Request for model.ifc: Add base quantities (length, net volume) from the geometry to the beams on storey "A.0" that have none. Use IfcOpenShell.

First a look at what the model holds.

```python
import ifcopenshell
import ifcopenshell.util.element
import ifcopenshell.util.unit

model = ifcopenshell.open("model.ifc")
print(model.schema)
for unit_type in ("LENGTHUNIT", "AREAUNIT", "VOLUMEUNIT"):
    print(unit_type, ifcopenshell.util.unit.calculate_unit_scale(model, unit_type))
storey = next(s for s in model.by_type("IfcBuildingStorey") if s.Name == "A.0")
beams = [e for e in ifcopenshell.util.element.get_decomposition(storey) if e.is_a("IfcBeam")]
for e in sorted(beams, key=lambda e: e.id()):
    print(e.id(), e.is_a(), e.Name, list(ifcopenshell.util.element.get_psets(e, qtos_only=True)), sep=" | ")
```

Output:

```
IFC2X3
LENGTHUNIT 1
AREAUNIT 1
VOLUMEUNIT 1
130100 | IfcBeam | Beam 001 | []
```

```python
import ifcopenshell
import ifcopenshell.api.pset
import ifcopenshell.geom
import ifcopenshell.util.element
import ifcopenshell.util.shape
import ifcopenshell.util.unit

model = ifcopenshell.open("model.ifc")
unit_scale = ifcopenshell.util.unit.calculate_unit_scale(model)
volume_scale = ifcopenshell.util.unit.calculate_unit_scale(model, "VOLUMEUNIT")
settings = ifcopenshell.geom.settings()

storey = next(s for s in model.by_type("IfcBuildingStorey") if s.Name == "A.0")
beams = [e for e in ifcopenshell.util.element.get_decomposition(storey) if e.is_a("IfcBeam")]

for e in sorted(beams, key=lambda e: e.id()):
    if ifcopenshell.util.element.get_psets(e, qtos_only=True, should_inherit=False):
        continue
    # Geometry comes back in metres, in the element's own axes.
    shape = ifcopenshell.geom.create_shape(settings, e)
    values = {
        "Length": ifcopenshell.util.shape.get_max_xyz(shape.geometry) / unit_scale,
        "NetVolume": ifcopenshell.util.shape.get_volume(shape.geometry) / volume_scale,
    }
    qto = ifcopenshell.api.pset.add_qto(model, product=e, name="BaseQuantities")
    ifcopenshell.api.pset.edit_qto(model, qto=qto, properties=values)
    print(e.id(), {k: round(v, 3) for k, v in values.items()})

model.write("model_rev.ifc")
```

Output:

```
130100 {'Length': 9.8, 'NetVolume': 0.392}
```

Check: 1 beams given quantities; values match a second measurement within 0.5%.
